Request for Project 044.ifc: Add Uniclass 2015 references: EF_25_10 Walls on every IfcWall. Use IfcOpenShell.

First a look at what the model holds.

```python
import ifcopenshell

model = ifcopenshell.open("Project 044.ifc")
print(model.schema)
print("classifications:", [c.Name for c in model.by_type("IfcClassification")])
for ifc_class in ("IfcDoor", "IfcRoof", "IfcStair", "IfcWall", "IfcWindow"):
    print(ifc_class, len(model.by_type(ifc_class)))
```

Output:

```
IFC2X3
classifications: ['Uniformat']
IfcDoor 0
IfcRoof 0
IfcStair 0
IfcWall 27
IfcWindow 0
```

```python
import ifcopenshell
import ifcopenshell.api.classification

model = ifcopenshell.open("Project 044.ifc")

# IFC2X3 requires Source and Edition and has no link from the project to the system.
system = model.create_entity("IfcClassification", Source="NBS", Edition="2015", Name="Uniclass 2015")

codes = {
    "IfcWall": ("EF_25_10", "Walls"),
}
for ifc_class, (code, name) in codes.items():
    products = model.by_type(ifc_class)
    ifcopenshell.api.classification.add_reference(
        model, products=products, classification=system, identification=code, name=name
    )
    print(code, len(products))

model.write("Project 044-out.ifc")
```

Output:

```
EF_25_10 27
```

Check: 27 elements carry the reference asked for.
